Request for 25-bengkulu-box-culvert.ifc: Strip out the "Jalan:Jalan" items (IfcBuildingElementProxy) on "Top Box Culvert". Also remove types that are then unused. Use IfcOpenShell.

First a look at what the model holds.

```python
import ifcopenshell
import ifcopenshell.util.element

model = ifcopenshell.open("25-bengkulu-box-culvert.ifc")
print(model.schema)
storey = next(s for s in model.by_type("IfcBuildingStorey") if s.Name == "Top Box Culvert")
proxies = [e for e in ifcopenshell.util.element.get_decomposition(storey) if e.is_a("IfcBuildingElementProxy")]
seen = {}
for e in proxies:
    element_type = ifcopenshell.util.element.get_type(e)
    name = element_type.Name if element_type not in (None, e) else None
    seen[name] = seen.get(name, 0) + 1
for name, count in sorted(seen.items(), key=str):
    print(count, "x", name)
```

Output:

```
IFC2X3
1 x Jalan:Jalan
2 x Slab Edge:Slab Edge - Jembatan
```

```python
import ifcopenshell
import ifcopenshell.api.root
import ifcopenshell.util.element

model = ifcopenshell.open("25-bengkulu-box-culvert.ifc")

storey = next(s for s in model.by_type("IfcBuildingStorey") if s.Name == "Top Box Culvert")
proxies = [e for e in ifcopenshell.util.element.get_decomposition(storey) if e.is_a("IfcBuildingElementProxy")]
targets = [e for e in proxies if (t := ifcopenshell.util.element.get_type(e)) not in (None, e) and t.Name == "Jalan:Jalan"]
types = {ifcopenshell.util.element.get_type(e) for e in targets} - {None, *targets}

for e in targets:
    ifcopenshell.api.root.remove_product(model, product=e)
print(len(targets), "removed")

unused = [t for t in types if not ifcopenshell.util.element.get_types(t)]
for t in unused:
    ifcopenshell.api.root.remove_product(model, product=t)
print(len(unused), "unused types removed")

model.write("25-bengkulu-box-culvert_v2.ifc")
```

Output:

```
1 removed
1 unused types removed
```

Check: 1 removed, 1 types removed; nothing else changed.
